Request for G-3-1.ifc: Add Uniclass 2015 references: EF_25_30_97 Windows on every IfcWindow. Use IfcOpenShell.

First a look at what the model holds.

```python
import ifcopenshell

model = ifcopenshell.open("G-3-1.ifc")
print(model.schema)
print("classifications:", [c.Name for c in model.by_type("IfcClassification")])
for ifc_class in ("IfcDoor", "IfcRoof", "IfcStair", "IfcWall", "IfcWindow"):
    print(ifc_class, len(model.by_type(ifc_class)))
```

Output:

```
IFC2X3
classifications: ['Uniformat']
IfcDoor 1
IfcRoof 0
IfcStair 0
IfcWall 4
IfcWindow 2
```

```python
import ifcopenshell
import ifcopenshell.api.classification

model = ifcopenshell.open("G-3-1.ifc")

# IFC2X3 requires Source and Edition and has no link from the project to the system.
system = model.create_entity("IfcClassification", Source="NBS", Edition="2015", Name="Uniclass 2015")

codes = {
    "IfcWindow": ("EF_25_30_97", "Windows"),
}
for ifc_class, (code, name) in codes.items():
    products = model.by_type(ifc_class)
    ifcopenshell.api.classification.add_reference(
        model, products=products, classification=system, identification=code, name=name
    )
    print(code, len(products))

model.write("G-3-1_v2.ifc")
```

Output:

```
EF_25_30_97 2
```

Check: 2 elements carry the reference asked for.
